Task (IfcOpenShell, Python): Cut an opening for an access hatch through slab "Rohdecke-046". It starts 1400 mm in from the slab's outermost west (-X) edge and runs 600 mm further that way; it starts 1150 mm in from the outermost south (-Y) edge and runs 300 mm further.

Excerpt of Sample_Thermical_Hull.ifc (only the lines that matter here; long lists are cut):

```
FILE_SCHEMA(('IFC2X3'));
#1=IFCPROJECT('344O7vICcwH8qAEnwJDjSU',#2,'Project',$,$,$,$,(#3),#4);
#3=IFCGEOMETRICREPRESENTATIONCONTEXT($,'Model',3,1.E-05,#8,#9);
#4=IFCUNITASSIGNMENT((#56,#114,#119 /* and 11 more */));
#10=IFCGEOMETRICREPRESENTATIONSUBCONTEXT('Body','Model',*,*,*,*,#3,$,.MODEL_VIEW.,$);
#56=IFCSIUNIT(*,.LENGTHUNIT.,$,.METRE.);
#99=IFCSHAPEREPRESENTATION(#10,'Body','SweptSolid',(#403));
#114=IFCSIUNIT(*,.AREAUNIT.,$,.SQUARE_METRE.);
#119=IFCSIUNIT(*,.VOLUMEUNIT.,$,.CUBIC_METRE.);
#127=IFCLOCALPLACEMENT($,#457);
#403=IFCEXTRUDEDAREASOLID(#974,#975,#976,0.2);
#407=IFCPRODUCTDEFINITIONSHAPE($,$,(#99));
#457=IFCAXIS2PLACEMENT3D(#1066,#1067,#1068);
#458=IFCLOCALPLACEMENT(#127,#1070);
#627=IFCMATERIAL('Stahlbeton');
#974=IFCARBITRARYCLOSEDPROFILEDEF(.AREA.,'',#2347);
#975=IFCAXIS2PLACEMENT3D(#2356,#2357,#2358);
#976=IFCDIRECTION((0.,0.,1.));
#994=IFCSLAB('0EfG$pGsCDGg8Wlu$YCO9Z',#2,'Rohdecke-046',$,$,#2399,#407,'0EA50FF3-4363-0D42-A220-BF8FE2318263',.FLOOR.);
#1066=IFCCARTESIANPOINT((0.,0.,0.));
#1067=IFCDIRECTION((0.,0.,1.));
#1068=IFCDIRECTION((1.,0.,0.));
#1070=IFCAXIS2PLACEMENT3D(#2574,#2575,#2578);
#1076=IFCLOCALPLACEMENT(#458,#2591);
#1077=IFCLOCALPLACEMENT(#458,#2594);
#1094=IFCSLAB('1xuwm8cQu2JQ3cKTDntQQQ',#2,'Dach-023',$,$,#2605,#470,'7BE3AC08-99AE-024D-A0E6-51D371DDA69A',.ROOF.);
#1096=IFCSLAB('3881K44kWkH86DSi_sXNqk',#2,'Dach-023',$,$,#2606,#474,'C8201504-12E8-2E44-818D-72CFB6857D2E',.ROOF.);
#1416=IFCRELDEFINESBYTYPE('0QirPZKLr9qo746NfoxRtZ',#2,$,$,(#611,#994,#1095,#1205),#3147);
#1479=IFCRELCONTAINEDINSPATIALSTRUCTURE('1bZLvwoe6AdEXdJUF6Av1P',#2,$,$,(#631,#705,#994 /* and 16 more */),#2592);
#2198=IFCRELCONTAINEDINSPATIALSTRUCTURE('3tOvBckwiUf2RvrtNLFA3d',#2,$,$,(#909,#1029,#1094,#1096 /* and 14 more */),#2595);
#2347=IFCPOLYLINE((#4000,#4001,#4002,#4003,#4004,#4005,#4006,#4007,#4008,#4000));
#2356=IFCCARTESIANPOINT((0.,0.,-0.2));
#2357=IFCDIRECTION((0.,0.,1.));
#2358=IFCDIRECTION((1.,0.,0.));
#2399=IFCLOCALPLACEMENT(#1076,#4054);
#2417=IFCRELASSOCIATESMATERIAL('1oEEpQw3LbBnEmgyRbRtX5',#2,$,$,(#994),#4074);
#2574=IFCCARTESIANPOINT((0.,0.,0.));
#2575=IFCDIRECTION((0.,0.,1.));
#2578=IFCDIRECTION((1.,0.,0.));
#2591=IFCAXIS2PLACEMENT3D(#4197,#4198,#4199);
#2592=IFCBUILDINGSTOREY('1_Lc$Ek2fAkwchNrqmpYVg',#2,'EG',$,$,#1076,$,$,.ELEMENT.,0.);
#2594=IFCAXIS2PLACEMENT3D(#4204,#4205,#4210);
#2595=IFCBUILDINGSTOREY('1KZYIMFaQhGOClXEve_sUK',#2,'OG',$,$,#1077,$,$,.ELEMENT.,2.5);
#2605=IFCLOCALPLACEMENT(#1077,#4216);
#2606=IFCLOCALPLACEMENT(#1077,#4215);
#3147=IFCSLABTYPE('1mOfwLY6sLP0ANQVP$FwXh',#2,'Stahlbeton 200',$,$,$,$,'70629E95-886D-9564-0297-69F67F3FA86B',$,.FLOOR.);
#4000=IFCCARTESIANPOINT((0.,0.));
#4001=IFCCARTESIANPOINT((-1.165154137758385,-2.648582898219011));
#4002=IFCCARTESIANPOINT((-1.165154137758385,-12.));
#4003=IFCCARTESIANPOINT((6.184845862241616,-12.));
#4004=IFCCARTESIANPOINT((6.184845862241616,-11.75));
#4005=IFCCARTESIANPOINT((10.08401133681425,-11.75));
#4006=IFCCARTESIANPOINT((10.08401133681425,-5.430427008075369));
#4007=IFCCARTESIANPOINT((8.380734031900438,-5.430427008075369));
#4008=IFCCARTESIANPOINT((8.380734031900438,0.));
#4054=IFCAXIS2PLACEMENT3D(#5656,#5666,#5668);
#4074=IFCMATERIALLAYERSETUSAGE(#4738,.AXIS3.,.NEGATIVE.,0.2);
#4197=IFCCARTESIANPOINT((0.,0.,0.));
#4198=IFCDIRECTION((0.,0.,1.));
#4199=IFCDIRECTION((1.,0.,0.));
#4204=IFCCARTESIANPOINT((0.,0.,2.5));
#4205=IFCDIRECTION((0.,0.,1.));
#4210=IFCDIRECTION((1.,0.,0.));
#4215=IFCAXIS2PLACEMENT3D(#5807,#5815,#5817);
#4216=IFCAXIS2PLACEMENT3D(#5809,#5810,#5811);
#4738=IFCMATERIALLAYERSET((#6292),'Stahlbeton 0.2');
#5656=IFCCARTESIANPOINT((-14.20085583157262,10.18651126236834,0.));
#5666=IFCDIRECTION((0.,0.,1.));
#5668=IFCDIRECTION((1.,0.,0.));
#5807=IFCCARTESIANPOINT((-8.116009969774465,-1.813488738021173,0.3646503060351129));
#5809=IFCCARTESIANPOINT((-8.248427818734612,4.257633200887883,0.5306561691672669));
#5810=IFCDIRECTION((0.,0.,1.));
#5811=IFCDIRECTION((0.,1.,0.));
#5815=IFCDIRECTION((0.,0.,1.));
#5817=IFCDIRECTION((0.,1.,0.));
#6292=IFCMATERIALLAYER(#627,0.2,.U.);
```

```python
import numpy as np
import ifcopenshell
import ifcopenshell.api.feature
import ifcopenshell.api.geometry
import ifcopenshell.api.root
import ifcopenshell.geom
import ifcopenshell.util.placement
import ifcopenshell.util.representation
import ifcopenshell.util.shape
import ifcopenshell.util.unit

model = ifcopenshell.open("Sample_Thermical_Hull.ifc")
unit_scale = ifcopenshell.util.unit.calculate_unit_scale(model)
settings = ifcopenshell.geom.settings()


def volume(element):
    """Net volume in cubic metres, openings subtracted."""
    shape = ifcopenshell.geom.create_shape(settings, element)
    return ifcopenshell.util.shape.get_volume(shape.geometry)


slab = model.by_guid("0EfG$pGsCDGg8Wlu$YCO9Z")
before = volume(slab)

# Extent in the slab's own axes, in metres. The edges named are its -X and -Y sides.
slab_shape = ifcopenshell.geom.create_shape(settings, slab)
vertices = ifcopenshell.util.shape.get_vertices(slab_shape.geometry)
x_min, y_min, bottom = vertices.min(axis=0)
top = vertices[:, 2].max()

opening = ifcopenshell.api.root.create_entity(model, ifc_class="IfcOpeningElement", name="Access hatch opening")
context = ifcopenshell.util.representation.get_context(model, "Model", "Body", "MODEL_VIEW")
width, depth = 0.6, 0.3
outline = [(0.0, 0.0), (width, 0.0), (width, depth), (0.0, depth), (0.0, 0.0)]
# Overshoot both faces by 50 mm so the cut is clean.
shape = ifcopenshell.api.geometry.add_slab_representation(
    model, context=context, depth=top - bottom + 0.1, polyline=outline
)
ifcopenshell.api.geometry.assign_representation(model, product=opening, representation=shape)

matrix = ifcopenshell.util.placement.get_local_placement(slab.ObjectPlacement)
matrix[:, 3] = matrix @ np.append(np.array([x_min + 1.4, y_min + 1.15, bottom - 0.05]) / unit_scale, 1.0)
ifcopenshell.api.geometry.edit_object_placement(model, product=opening, matrix=matrix, is_si=False)
ifcopenshell.api.feature.add_feature(model, feature=opening, element=slab)

after = volume(slab)

print(f"slab volume {before:.3f} -> {after:.3f} m3")

model.write("Sample_Thermical_Hull_rev.ifc")
```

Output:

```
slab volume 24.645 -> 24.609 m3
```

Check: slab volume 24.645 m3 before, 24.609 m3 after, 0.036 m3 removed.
